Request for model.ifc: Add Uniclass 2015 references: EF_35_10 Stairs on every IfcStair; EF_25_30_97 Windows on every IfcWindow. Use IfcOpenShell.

First a look at what the model holds.

```python
import ifcopenshell

model = ifcopenshell.open("model.ifc")
print(model.schema)
print("classifications:", [c.Name for c in model.by_type("IfcClassification")])
for ifc_class in ("IfcDoor", "IfcRoof", "IfcStair", "IfcWall", "IfcWindow"):
    print(ifc_class, len(model.by_type(ifc_class)))
```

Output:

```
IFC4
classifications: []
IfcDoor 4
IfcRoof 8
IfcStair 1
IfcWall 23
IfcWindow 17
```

```python
import ifcopenshell
import ifcopenshell.api.classification

model = ifcopenshell.open("model.ifc")

system = ifcopenshell.api.classification.add_classification(model, classification="Uniclass 2015")

codes = {
    "IfcStair": ("EF_35_10", "Stairs"),
    "IfcWindow": ("EF_25_30_97", "Windows"),
}
for ifc_class, (code, name) in codes.items():
    products = model.by_type(ifc_class)
    ifcopenshell.api.classification.add_reference(
        model, products=products, classification=system, identification=code, name=name
    )
    print(code, len(products))

model.write("model_edited.ifc")
```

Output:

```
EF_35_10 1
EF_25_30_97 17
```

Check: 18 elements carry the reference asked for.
